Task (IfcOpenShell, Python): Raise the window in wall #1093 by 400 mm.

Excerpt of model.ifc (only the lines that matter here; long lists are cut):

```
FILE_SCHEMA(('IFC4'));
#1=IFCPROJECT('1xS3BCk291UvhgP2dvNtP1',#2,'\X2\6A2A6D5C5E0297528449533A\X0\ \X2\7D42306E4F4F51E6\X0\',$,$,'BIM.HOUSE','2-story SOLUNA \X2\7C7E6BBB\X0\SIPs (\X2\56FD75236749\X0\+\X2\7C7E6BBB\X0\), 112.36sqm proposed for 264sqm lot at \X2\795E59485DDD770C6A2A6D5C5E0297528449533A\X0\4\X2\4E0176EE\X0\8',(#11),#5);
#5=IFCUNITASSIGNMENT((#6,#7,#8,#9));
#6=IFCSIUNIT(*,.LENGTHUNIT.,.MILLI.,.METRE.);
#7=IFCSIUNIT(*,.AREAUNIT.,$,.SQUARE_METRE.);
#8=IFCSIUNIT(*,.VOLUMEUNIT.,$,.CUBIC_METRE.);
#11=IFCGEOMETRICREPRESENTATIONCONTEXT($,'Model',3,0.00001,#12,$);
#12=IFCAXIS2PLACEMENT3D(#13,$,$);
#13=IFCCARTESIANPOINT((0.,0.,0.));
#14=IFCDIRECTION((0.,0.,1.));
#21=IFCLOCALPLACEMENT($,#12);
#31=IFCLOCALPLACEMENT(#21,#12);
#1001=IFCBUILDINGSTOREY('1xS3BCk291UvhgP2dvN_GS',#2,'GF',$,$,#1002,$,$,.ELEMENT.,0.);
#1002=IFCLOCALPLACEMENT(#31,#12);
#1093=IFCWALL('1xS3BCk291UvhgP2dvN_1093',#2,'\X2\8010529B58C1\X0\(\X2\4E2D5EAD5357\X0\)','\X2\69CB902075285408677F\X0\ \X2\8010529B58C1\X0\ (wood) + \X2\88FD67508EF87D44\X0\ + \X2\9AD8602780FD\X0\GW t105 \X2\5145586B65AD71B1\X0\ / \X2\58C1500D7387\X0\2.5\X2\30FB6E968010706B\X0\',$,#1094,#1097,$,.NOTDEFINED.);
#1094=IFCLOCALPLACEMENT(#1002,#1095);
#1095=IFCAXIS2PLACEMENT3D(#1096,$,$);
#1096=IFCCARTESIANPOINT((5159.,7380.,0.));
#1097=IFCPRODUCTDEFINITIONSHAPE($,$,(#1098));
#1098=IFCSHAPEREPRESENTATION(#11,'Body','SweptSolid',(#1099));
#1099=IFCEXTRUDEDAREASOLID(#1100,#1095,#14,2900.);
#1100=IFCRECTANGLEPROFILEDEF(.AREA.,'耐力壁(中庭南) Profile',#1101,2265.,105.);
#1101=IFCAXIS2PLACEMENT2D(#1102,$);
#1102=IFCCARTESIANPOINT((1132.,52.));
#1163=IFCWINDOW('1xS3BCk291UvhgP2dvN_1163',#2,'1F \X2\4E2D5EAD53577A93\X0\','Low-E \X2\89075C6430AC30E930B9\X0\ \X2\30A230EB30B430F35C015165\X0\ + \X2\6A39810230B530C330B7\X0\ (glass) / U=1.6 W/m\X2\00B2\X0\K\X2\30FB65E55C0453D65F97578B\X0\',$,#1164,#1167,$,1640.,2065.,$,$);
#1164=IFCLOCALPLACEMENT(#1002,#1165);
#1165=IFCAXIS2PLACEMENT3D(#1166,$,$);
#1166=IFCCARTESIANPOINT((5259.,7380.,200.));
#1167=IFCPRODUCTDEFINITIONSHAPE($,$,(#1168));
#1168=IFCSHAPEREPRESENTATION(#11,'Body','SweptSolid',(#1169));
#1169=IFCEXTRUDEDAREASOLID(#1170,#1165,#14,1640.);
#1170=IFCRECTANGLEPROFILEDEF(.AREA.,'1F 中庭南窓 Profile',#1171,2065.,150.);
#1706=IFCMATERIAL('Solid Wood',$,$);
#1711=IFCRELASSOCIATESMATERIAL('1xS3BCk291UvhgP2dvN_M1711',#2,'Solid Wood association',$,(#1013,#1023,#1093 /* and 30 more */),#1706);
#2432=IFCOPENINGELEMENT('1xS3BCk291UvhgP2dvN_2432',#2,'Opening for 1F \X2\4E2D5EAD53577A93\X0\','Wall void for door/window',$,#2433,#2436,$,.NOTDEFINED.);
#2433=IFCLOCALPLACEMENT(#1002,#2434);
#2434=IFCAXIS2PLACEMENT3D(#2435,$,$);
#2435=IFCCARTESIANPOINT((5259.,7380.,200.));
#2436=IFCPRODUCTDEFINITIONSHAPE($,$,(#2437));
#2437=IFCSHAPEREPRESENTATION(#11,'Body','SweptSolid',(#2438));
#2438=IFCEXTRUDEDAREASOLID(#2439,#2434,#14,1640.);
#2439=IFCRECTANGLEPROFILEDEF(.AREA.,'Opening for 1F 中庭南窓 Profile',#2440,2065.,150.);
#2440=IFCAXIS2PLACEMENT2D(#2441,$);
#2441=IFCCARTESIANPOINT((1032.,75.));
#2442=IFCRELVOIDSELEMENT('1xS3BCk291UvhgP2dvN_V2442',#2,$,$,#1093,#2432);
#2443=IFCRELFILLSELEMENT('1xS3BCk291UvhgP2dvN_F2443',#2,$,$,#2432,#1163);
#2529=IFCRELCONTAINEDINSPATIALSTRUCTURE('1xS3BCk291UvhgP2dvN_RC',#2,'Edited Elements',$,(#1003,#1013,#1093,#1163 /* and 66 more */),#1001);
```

```python
import numpy as np
import ifcopenshell
import ifcopenshell.api.geometry
import ifcopenshell.util.placement
import ifcopenshell.util.unit

model = ifcopenshell.open("model.ifc")
unit_scale = ifcopenshell.util.unit.calculate_unit_scale(model)

window = model.by_guid("1xS3BCk291UvhgP2dvN_1163")
opening = window.FillsVoids[0].RelatingOpeningElement
dz = 0.4 / unit_scale

shift = np.array([0.0, 0.0, dz])
# The window is not placed relative to its opening, so move both.
for product in (opening, window):
    matrix = ifcopenshell.util.placement.get_local_placement(product.ObjectPlacement)
    matrix[:3, 3] += shift
    ifcopenshell.api.geometry.edit_object_placement(model, product=product, matrix=matrix, is_si=False)

print(f"moved by {dz * unit_scale:+.3f} m")

model.write("model-out.ifc")
```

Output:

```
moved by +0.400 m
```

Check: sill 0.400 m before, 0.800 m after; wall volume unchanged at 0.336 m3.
